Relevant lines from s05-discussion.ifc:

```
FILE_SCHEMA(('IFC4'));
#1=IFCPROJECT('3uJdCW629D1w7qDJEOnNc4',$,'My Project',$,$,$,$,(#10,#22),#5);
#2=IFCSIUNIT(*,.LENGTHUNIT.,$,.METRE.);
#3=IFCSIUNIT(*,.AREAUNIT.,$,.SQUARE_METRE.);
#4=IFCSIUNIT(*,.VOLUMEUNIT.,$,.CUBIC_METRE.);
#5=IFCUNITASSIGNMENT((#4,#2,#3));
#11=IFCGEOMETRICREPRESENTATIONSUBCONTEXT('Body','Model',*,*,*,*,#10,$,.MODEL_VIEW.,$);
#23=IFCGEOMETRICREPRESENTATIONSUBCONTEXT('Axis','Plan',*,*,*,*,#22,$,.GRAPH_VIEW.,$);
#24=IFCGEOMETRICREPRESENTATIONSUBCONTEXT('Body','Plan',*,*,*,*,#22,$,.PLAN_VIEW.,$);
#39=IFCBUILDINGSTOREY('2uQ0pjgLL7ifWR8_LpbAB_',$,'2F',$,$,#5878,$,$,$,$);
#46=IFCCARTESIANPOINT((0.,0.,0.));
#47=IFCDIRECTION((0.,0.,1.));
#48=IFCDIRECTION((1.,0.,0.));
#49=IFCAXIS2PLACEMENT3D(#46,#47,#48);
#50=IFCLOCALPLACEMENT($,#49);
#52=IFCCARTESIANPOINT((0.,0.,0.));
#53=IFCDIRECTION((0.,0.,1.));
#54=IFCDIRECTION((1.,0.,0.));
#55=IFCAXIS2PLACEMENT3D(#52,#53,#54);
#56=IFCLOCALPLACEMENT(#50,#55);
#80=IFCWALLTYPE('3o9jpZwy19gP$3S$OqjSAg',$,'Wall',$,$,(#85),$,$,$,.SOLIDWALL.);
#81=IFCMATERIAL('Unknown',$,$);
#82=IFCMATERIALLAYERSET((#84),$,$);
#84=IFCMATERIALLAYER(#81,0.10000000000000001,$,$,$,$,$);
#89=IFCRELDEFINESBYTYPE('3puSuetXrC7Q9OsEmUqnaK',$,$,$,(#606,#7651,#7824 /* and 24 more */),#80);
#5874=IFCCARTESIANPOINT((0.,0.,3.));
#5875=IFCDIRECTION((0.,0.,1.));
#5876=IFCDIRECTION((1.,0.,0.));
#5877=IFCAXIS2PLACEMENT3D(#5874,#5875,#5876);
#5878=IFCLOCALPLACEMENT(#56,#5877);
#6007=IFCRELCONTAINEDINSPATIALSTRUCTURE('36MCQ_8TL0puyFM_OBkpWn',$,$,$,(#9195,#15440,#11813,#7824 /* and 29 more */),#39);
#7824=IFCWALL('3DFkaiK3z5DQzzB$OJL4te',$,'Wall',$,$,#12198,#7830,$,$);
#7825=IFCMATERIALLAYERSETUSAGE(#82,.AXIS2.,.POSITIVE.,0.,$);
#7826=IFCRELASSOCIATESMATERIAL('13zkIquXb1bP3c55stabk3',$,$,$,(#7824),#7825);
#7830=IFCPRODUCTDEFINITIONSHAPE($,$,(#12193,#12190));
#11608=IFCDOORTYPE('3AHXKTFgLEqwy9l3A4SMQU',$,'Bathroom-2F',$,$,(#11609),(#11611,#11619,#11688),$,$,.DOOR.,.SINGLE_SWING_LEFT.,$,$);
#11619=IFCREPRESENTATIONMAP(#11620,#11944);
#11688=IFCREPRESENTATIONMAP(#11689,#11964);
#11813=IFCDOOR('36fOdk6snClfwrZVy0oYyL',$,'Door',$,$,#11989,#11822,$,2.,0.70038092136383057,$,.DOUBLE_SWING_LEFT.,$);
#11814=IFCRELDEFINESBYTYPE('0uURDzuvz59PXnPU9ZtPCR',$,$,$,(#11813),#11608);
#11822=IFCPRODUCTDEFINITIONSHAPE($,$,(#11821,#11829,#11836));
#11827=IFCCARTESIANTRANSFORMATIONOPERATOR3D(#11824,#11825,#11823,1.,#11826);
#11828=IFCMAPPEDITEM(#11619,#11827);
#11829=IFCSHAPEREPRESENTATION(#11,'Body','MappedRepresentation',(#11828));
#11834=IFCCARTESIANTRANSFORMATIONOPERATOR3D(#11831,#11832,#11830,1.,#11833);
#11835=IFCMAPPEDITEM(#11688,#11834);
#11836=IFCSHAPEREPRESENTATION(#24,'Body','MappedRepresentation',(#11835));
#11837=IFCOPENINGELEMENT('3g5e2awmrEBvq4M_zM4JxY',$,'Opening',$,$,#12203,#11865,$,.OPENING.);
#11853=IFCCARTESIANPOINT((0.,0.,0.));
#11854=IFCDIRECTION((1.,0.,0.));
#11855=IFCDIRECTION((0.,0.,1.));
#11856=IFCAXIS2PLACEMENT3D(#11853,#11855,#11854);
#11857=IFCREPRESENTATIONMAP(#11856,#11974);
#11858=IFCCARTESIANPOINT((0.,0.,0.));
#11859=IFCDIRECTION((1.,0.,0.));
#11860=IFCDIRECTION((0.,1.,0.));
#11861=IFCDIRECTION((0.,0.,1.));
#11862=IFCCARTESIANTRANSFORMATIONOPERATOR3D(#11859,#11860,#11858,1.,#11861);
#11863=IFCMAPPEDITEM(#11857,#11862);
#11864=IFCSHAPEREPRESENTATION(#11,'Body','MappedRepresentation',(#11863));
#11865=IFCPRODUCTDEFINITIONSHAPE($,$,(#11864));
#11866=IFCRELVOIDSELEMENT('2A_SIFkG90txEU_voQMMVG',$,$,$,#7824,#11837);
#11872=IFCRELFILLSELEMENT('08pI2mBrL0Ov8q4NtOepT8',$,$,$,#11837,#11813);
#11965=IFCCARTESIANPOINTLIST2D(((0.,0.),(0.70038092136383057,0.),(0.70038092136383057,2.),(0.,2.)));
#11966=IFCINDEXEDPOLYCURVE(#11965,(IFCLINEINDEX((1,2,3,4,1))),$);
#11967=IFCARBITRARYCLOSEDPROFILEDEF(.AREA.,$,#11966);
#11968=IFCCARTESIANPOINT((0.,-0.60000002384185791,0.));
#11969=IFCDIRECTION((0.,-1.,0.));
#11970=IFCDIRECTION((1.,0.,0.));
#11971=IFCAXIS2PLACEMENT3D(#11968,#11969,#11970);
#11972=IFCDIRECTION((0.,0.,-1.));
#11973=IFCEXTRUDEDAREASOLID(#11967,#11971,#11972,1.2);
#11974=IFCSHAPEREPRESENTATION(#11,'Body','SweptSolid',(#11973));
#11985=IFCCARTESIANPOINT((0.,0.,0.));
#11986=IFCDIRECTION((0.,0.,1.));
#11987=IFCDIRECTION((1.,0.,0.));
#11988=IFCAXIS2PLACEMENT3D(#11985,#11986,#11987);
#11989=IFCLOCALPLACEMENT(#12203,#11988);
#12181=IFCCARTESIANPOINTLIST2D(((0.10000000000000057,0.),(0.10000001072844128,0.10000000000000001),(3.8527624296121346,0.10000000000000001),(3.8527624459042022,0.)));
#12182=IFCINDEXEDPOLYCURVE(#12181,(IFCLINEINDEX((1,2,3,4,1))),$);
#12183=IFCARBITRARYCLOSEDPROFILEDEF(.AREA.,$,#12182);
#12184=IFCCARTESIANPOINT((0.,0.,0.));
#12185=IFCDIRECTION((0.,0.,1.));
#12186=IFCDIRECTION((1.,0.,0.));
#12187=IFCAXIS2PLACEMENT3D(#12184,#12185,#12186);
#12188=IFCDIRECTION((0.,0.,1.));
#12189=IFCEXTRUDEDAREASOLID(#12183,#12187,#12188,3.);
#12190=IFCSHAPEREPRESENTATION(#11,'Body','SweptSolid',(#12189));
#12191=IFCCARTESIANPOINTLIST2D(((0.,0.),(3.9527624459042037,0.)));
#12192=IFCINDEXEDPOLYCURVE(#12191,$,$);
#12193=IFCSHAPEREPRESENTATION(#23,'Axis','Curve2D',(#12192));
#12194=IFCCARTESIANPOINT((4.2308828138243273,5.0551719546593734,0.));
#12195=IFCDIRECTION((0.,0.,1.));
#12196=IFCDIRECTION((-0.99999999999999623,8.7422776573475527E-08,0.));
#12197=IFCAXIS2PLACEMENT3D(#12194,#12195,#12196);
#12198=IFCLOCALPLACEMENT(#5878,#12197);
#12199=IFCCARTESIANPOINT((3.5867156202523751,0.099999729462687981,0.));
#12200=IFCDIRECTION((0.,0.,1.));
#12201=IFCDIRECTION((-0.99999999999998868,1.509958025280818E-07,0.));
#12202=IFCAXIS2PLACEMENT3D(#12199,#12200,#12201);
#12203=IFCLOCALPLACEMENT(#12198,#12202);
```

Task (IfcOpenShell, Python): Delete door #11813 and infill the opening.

```python
import ifcopenshell
import ifcopenshell.api.feature
import ifcopenshell.api.root
import ifcopenshell.geom
import ifcopenshell.util.shape

model = ifcopenshell.open("s05-discussion.ifc")
settings = ifcopenshell.geom.settings()


def volume(element):
    """Net volume in cubic metres, openings subtracted."""
    shape = ifcopenshell.geom.create_shape(settings, element)
    return ifcopenshell.util.shape.get_volume(shape.geometry)


door = model.by_guid("36fOdk6snClfwrZVy0oYyL")
opening = door.FillsVoids[0].RelatingOpeningElement
wall = opening.VoidsElements[0].RelatingBuildingElement
before = volume(wall)

ifcopenshell.api.root.remove_product(model, product=door)
ifcopenshell.api.feature.remove_feature(model, feature=opening)

after = volume(wall)

print(f"wall volume {before:.3f} -> {after:.3f} m3")

model.write("s05-discussion_edited.ifc")
```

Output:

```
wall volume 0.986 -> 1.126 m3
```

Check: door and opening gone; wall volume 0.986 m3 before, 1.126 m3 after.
